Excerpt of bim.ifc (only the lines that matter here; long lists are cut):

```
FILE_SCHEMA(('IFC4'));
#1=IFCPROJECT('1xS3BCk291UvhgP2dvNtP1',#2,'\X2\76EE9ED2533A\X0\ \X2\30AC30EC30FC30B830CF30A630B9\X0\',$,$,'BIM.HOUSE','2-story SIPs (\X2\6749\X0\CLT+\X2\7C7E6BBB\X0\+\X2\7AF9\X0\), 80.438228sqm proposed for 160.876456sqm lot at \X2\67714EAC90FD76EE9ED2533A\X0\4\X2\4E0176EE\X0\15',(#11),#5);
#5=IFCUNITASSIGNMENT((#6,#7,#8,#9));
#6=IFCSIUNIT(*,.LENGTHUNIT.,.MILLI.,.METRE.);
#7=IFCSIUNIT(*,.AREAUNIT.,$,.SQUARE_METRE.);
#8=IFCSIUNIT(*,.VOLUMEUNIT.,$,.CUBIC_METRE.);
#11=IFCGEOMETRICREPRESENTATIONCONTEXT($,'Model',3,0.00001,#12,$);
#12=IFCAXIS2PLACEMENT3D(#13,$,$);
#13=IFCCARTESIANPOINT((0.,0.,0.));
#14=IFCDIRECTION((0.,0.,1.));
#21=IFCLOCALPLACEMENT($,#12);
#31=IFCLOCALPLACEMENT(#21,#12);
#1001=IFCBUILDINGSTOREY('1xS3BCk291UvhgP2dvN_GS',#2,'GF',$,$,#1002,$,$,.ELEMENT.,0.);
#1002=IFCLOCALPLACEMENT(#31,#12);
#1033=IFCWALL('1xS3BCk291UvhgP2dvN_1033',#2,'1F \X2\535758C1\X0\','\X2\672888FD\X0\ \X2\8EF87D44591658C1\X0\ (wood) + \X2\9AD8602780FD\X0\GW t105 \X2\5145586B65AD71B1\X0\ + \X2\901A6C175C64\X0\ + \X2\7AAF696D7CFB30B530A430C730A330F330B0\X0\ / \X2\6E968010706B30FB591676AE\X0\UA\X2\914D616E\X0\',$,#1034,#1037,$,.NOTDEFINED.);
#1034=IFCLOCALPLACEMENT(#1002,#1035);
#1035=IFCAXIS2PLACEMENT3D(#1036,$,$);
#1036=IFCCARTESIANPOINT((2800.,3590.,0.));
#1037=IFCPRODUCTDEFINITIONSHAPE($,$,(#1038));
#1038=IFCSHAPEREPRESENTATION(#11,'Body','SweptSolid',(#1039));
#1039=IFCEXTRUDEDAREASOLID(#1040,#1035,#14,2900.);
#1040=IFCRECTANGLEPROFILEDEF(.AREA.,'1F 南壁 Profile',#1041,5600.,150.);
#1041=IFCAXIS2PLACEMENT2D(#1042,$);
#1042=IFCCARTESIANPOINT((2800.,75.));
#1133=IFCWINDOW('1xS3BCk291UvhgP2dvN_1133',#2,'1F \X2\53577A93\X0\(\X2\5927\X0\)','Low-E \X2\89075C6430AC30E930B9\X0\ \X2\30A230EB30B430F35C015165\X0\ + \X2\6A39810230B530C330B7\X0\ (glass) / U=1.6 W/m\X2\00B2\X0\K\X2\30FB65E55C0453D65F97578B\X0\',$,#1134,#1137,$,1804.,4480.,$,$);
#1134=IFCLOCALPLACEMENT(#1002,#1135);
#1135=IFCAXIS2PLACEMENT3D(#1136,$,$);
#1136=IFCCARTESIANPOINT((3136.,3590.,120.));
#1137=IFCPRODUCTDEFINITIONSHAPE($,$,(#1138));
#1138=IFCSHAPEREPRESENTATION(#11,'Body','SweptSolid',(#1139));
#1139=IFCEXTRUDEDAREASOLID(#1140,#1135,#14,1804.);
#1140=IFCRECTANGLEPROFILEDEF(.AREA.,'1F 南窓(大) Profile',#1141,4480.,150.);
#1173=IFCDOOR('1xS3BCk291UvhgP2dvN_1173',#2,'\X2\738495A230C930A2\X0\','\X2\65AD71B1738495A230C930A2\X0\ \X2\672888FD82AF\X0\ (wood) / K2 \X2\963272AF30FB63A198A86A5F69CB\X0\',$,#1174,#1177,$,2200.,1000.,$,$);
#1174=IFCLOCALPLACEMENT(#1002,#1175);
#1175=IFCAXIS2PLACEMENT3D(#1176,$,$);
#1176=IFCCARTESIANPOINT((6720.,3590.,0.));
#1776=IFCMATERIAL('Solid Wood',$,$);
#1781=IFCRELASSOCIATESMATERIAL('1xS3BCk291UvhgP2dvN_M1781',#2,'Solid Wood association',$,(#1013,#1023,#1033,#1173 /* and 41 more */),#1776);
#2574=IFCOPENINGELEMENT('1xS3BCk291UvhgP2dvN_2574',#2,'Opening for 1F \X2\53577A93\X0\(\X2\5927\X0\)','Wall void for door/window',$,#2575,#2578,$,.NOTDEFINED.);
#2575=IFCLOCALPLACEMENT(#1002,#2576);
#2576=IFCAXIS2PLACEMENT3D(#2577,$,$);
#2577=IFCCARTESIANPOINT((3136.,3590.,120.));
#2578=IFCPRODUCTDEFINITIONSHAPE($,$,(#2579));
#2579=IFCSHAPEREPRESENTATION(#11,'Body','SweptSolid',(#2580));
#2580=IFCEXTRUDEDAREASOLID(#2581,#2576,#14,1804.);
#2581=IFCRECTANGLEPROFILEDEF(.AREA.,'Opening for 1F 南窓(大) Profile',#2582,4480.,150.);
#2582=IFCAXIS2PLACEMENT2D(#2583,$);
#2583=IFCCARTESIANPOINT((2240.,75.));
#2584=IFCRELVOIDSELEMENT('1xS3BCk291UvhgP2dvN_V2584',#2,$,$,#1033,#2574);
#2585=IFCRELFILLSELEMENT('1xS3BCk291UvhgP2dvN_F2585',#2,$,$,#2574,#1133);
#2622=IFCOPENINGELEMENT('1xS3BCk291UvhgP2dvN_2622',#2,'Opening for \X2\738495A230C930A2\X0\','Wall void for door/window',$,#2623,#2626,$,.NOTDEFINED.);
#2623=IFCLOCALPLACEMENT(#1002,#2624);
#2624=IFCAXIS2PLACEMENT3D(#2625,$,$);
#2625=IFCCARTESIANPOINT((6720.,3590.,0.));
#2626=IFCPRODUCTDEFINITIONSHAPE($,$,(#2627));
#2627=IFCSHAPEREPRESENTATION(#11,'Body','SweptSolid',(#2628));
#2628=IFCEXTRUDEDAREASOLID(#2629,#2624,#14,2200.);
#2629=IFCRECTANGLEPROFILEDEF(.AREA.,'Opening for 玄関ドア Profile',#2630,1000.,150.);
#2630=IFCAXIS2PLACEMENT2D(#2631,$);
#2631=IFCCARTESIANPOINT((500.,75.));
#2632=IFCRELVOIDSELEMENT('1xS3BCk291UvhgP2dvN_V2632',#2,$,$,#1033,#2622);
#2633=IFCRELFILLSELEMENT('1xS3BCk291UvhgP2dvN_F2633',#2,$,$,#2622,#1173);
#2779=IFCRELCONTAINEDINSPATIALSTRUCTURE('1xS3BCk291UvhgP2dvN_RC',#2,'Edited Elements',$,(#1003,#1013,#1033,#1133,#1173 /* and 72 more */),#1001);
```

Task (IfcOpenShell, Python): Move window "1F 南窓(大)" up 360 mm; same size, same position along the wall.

```python
import numpy as np
import ifcopenshell
import ifcopenshell.api.geometry
import ifcopenshell.util.placement
import ifcopenshell.util.unit

model = ifcopenshell.open("bim.ifc")
unit_scale = ifcopenshell.util.unit.calculate_unit_scale(model)

window = model.by_guid("1xS3BCk291UvhgP2dvN_1133")
opening = window.FillsVoids[0].RelatingOpeningElement
dz = 0.36 / unit_scale

shift = np.array([0.0, 0.0, dz])
# The window is not placed relative to its opening, so move both.
for product in (opening, window):
    matrix = ifcopenshell.util.placement.get_local_placement(product.ObjectPlacement)
    matrix[:3, 3] += shift
    ifcopenshell.api.geometry.edit_object_placement(model, product=product, matrix=matrix, is_si=False)

print(f"moved by {dz * unit_scale:+.3f} m")

model.write("bim_rev.ifc")
```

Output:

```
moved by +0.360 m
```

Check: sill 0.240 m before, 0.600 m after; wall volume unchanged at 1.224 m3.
